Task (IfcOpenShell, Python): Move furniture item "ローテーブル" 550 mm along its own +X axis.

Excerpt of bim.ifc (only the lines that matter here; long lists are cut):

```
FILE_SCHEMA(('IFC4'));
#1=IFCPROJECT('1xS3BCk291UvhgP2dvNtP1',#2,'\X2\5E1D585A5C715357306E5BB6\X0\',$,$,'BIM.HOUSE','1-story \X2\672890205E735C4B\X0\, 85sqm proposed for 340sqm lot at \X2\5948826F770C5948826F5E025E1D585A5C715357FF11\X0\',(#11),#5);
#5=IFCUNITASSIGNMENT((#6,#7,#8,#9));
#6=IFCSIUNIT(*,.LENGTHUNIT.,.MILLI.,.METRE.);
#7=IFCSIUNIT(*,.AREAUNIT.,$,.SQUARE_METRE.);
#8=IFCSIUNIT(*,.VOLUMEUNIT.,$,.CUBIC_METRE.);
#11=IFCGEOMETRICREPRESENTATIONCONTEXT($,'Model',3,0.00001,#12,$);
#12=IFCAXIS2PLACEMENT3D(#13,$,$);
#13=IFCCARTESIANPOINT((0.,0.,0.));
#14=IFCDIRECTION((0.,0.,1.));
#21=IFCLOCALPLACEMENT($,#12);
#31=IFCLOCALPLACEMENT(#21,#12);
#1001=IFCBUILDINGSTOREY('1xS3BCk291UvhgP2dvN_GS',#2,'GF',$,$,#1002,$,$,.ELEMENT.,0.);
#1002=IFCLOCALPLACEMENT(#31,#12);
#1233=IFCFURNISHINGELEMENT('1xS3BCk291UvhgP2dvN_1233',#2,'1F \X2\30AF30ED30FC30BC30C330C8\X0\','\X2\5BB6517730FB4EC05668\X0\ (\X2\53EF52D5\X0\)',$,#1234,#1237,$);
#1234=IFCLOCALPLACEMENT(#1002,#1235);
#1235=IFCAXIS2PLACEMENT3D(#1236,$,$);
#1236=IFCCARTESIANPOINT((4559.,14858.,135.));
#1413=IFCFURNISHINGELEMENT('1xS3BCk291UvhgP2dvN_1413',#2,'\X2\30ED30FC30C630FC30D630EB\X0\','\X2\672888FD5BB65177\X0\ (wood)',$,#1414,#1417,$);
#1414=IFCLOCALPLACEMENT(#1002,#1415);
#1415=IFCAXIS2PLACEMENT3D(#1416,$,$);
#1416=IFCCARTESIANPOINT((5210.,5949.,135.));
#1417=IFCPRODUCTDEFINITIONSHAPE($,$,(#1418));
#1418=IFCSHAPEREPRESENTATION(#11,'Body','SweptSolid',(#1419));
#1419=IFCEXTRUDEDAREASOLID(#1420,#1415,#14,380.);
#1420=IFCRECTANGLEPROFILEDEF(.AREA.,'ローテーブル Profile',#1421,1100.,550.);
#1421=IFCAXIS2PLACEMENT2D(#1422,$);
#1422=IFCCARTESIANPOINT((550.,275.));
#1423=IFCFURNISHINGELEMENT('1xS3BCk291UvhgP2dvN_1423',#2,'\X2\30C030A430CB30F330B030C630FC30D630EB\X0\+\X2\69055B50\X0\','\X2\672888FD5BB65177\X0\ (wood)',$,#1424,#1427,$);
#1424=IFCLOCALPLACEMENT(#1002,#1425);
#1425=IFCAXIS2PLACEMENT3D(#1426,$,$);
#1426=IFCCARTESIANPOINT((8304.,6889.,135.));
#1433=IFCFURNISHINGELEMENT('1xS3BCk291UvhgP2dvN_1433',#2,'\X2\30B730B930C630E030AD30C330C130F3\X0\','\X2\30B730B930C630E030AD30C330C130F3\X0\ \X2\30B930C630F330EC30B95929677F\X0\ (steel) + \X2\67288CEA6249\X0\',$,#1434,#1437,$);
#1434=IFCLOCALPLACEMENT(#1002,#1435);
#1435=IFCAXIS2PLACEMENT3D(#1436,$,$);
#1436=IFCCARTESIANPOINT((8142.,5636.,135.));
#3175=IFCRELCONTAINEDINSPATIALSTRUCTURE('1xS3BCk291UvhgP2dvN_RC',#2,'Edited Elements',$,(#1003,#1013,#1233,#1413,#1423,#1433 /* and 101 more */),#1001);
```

```python
import ifcopenshell
import ifcopenshell.api.geometry
import ifcopenshell.util.placement
import ifcopenshell.util.unit

model = ifcopenshell.open("bim.ifc")
unit_scale = ifcopenshell.util.unit.calculate_unit_scale(model)

item = model.by_guid("1xS3BCk291UvhgP2dvN_1413")
matrix = ifcopenshell.util.placement.get_local_placement(item.ObjectPlacement)
matrix[:3, 3] += matrix[:3, 0] * 0.55 / unit_scale
ifcopenshell.api.geometry.edit_object_placement(model, product=item, matrix=matrix, is_si=False)

print(ifcopenshell.util.placement.get_local_placement(item.ObjectPlacement).round(3) + 0.0)

model.write("bim_v2.ifc")
```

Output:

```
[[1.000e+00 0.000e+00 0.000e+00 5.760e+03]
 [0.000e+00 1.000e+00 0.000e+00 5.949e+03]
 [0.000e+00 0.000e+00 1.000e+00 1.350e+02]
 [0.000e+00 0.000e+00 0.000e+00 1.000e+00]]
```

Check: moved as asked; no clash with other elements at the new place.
